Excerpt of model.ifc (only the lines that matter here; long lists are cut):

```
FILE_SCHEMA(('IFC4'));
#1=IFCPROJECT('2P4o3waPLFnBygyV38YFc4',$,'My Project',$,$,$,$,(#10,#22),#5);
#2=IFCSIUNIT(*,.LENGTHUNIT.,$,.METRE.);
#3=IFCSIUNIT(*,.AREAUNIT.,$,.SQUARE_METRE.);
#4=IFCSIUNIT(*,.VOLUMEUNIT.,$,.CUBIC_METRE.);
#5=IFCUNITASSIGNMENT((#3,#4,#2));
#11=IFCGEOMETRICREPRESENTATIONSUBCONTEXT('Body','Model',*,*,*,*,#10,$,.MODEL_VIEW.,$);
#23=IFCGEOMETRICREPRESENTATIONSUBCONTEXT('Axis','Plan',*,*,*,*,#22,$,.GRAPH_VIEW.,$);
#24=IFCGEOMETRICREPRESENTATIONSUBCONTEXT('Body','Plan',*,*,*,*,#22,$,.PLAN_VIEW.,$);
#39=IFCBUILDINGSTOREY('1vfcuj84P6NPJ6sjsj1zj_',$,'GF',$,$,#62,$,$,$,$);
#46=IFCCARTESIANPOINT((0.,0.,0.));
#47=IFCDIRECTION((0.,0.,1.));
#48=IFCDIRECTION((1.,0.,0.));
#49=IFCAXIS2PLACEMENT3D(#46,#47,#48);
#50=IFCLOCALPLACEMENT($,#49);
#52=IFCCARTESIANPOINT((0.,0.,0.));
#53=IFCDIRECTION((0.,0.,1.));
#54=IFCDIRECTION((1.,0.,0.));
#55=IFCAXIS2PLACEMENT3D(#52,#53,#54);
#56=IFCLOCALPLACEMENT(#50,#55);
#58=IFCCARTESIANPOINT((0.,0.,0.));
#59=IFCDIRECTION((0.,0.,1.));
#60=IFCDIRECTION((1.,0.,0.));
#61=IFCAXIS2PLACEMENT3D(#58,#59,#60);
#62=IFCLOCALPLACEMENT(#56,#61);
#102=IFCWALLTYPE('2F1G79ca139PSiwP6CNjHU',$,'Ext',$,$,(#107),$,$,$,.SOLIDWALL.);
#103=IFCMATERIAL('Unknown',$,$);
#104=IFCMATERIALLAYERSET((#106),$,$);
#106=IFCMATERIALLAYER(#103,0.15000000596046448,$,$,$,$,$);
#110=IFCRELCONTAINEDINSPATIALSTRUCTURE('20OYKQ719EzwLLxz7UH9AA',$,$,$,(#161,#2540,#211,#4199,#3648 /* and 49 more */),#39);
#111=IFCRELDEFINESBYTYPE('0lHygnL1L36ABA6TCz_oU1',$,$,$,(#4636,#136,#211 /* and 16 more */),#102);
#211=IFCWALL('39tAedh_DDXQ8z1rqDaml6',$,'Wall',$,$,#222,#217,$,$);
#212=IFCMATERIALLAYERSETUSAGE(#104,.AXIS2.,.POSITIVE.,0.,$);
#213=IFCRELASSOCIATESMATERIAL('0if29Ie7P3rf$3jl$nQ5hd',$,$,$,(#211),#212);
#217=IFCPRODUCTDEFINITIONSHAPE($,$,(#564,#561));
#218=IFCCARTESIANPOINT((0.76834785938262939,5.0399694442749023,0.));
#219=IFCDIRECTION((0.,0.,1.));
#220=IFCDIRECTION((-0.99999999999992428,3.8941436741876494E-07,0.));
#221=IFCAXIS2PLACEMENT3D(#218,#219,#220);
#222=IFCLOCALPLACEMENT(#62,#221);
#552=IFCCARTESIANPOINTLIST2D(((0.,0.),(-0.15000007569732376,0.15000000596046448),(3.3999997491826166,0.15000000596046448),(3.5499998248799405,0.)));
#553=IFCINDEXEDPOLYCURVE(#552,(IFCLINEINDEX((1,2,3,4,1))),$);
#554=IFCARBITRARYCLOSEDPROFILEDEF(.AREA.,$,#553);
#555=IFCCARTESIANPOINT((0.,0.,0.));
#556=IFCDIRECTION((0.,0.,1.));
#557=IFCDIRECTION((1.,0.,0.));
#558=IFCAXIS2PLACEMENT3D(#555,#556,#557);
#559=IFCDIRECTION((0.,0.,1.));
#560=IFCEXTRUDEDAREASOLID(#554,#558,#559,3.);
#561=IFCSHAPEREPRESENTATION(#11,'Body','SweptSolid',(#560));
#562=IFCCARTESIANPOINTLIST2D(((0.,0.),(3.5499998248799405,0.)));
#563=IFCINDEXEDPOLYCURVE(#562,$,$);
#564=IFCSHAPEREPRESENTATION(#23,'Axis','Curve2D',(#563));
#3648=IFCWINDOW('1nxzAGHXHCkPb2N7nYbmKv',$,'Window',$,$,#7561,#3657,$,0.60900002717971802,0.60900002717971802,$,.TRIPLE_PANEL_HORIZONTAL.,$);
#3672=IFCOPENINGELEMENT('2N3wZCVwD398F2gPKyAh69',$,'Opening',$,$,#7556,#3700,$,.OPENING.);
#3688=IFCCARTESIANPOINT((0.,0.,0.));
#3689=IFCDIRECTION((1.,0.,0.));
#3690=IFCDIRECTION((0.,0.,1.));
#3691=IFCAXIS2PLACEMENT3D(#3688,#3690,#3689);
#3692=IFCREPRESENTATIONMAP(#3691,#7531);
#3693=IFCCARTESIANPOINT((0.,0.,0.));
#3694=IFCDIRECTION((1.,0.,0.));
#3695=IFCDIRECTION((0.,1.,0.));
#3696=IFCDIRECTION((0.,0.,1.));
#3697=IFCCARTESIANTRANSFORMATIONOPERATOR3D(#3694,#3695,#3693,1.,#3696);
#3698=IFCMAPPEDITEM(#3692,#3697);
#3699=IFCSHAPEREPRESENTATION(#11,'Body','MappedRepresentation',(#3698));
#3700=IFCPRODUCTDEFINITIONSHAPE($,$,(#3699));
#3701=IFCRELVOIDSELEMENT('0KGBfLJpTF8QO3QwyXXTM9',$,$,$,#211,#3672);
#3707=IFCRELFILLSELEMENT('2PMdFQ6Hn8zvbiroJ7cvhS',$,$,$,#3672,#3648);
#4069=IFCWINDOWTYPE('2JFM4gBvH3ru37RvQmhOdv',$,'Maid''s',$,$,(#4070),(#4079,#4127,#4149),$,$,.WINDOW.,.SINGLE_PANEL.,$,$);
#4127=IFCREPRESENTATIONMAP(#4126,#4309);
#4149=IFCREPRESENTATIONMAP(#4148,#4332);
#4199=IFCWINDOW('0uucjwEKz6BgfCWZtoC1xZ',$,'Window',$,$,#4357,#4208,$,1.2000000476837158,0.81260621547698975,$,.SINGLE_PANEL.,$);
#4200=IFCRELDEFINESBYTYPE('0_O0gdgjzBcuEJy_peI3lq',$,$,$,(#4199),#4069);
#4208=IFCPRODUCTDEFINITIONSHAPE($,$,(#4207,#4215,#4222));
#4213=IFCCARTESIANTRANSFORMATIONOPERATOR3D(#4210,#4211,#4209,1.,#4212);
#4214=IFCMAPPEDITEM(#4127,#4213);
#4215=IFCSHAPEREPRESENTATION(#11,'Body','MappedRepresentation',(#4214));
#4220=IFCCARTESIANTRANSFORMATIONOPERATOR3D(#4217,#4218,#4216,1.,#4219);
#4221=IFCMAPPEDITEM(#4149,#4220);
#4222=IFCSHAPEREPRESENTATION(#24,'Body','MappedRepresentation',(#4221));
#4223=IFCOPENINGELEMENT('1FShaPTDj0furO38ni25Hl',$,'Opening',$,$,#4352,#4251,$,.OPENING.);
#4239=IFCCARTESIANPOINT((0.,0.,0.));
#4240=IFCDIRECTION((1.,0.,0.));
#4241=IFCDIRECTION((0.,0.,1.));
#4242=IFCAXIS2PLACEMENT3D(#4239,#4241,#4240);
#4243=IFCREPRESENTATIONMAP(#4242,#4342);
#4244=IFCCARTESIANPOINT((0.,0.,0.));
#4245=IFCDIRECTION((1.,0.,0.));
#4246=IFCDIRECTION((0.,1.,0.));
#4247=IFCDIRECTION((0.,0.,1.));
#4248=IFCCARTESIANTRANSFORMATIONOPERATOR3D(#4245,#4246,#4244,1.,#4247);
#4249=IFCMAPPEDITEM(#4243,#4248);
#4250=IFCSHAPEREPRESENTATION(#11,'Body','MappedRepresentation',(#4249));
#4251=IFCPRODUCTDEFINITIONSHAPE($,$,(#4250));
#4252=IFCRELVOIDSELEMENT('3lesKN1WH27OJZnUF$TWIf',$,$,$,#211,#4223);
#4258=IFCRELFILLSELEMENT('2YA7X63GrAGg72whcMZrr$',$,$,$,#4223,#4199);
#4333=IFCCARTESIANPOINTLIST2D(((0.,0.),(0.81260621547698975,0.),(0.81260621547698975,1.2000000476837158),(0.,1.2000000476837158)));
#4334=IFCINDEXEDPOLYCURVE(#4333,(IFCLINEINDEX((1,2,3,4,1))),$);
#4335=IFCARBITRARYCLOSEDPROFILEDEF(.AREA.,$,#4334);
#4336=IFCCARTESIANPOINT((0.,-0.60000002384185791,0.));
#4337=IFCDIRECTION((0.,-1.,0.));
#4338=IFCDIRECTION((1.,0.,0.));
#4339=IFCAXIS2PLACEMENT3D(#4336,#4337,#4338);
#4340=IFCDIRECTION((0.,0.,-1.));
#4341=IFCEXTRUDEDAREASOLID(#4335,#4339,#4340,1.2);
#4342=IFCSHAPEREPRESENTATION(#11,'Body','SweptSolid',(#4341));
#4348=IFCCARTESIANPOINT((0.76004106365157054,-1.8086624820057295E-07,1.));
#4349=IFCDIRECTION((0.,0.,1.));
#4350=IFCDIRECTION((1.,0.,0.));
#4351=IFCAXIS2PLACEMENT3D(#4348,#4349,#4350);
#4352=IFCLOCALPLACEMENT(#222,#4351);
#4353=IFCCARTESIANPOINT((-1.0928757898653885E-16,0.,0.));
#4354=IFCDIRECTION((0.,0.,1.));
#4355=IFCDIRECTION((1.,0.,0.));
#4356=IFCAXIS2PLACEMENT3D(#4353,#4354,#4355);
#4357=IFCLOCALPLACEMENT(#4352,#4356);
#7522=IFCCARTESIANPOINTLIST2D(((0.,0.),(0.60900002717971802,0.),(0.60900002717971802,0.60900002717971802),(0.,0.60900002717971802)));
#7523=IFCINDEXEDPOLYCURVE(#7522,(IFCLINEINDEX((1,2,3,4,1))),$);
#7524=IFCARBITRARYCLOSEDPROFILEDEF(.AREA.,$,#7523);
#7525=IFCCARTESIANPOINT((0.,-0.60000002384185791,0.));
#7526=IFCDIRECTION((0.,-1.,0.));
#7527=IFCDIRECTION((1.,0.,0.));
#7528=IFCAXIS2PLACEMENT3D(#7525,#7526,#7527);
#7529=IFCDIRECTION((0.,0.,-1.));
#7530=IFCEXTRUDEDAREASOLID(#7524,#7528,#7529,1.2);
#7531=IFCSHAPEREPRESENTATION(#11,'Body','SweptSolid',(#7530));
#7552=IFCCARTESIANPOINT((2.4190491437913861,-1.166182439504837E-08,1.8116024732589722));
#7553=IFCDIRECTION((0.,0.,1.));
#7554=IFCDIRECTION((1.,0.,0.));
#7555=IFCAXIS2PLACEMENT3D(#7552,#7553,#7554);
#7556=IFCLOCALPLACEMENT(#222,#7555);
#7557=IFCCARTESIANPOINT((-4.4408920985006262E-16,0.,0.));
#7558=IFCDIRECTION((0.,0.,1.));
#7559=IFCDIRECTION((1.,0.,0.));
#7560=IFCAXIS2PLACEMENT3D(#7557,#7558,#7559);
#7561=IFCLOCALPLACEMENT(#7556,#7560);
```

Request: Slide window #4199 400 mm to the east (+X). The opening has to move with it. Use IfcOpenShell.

```python
import ifcopenshell
import ifcopenshell.api.geometry
import ifcopenshell.util.placement

model = ifcopenshell.open("model.ifc")

window = model.by_guid("0uucjwEKz6BgfCWZtoC1xZ")
opening = window.FillsVoids[0].RelatingOpeningElement
wall = opening.VoidsElements[0].RelatingBuildingElement

wall_matrix = ifcopenshell.util.placement.get_local_placement(wall.ObjectPlacement)
shift = wall_matrix[:3, 0] * -0.4
before = ifcopenshell.util.placement.get_local_placement(window.ObjectPlacement)[:3, 3].copy()

# The window is placed relative to its opening, so it follows when the opening moves.
matrix = ifcopenshell.util.placement.get_local_placement(opening.ObjectPlacement)
matrix[:3, 3] += shift
ifcopenshell.api.geometry.edit_object_placement(
    model, product=opening, matrix=matrix, is_si=False, should_transform_children=True
)

after = ifcopenshell.util.placement.get_local_placement(window.ObjectPlacement)[:3, 3]
print("window moved by", (after - before).round(3) + 0.0)

model.write("model_v2.ifc")
```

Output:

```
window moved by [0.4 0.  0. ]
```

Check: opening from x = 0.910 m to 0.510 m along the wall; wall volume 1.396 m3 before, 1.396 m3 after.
